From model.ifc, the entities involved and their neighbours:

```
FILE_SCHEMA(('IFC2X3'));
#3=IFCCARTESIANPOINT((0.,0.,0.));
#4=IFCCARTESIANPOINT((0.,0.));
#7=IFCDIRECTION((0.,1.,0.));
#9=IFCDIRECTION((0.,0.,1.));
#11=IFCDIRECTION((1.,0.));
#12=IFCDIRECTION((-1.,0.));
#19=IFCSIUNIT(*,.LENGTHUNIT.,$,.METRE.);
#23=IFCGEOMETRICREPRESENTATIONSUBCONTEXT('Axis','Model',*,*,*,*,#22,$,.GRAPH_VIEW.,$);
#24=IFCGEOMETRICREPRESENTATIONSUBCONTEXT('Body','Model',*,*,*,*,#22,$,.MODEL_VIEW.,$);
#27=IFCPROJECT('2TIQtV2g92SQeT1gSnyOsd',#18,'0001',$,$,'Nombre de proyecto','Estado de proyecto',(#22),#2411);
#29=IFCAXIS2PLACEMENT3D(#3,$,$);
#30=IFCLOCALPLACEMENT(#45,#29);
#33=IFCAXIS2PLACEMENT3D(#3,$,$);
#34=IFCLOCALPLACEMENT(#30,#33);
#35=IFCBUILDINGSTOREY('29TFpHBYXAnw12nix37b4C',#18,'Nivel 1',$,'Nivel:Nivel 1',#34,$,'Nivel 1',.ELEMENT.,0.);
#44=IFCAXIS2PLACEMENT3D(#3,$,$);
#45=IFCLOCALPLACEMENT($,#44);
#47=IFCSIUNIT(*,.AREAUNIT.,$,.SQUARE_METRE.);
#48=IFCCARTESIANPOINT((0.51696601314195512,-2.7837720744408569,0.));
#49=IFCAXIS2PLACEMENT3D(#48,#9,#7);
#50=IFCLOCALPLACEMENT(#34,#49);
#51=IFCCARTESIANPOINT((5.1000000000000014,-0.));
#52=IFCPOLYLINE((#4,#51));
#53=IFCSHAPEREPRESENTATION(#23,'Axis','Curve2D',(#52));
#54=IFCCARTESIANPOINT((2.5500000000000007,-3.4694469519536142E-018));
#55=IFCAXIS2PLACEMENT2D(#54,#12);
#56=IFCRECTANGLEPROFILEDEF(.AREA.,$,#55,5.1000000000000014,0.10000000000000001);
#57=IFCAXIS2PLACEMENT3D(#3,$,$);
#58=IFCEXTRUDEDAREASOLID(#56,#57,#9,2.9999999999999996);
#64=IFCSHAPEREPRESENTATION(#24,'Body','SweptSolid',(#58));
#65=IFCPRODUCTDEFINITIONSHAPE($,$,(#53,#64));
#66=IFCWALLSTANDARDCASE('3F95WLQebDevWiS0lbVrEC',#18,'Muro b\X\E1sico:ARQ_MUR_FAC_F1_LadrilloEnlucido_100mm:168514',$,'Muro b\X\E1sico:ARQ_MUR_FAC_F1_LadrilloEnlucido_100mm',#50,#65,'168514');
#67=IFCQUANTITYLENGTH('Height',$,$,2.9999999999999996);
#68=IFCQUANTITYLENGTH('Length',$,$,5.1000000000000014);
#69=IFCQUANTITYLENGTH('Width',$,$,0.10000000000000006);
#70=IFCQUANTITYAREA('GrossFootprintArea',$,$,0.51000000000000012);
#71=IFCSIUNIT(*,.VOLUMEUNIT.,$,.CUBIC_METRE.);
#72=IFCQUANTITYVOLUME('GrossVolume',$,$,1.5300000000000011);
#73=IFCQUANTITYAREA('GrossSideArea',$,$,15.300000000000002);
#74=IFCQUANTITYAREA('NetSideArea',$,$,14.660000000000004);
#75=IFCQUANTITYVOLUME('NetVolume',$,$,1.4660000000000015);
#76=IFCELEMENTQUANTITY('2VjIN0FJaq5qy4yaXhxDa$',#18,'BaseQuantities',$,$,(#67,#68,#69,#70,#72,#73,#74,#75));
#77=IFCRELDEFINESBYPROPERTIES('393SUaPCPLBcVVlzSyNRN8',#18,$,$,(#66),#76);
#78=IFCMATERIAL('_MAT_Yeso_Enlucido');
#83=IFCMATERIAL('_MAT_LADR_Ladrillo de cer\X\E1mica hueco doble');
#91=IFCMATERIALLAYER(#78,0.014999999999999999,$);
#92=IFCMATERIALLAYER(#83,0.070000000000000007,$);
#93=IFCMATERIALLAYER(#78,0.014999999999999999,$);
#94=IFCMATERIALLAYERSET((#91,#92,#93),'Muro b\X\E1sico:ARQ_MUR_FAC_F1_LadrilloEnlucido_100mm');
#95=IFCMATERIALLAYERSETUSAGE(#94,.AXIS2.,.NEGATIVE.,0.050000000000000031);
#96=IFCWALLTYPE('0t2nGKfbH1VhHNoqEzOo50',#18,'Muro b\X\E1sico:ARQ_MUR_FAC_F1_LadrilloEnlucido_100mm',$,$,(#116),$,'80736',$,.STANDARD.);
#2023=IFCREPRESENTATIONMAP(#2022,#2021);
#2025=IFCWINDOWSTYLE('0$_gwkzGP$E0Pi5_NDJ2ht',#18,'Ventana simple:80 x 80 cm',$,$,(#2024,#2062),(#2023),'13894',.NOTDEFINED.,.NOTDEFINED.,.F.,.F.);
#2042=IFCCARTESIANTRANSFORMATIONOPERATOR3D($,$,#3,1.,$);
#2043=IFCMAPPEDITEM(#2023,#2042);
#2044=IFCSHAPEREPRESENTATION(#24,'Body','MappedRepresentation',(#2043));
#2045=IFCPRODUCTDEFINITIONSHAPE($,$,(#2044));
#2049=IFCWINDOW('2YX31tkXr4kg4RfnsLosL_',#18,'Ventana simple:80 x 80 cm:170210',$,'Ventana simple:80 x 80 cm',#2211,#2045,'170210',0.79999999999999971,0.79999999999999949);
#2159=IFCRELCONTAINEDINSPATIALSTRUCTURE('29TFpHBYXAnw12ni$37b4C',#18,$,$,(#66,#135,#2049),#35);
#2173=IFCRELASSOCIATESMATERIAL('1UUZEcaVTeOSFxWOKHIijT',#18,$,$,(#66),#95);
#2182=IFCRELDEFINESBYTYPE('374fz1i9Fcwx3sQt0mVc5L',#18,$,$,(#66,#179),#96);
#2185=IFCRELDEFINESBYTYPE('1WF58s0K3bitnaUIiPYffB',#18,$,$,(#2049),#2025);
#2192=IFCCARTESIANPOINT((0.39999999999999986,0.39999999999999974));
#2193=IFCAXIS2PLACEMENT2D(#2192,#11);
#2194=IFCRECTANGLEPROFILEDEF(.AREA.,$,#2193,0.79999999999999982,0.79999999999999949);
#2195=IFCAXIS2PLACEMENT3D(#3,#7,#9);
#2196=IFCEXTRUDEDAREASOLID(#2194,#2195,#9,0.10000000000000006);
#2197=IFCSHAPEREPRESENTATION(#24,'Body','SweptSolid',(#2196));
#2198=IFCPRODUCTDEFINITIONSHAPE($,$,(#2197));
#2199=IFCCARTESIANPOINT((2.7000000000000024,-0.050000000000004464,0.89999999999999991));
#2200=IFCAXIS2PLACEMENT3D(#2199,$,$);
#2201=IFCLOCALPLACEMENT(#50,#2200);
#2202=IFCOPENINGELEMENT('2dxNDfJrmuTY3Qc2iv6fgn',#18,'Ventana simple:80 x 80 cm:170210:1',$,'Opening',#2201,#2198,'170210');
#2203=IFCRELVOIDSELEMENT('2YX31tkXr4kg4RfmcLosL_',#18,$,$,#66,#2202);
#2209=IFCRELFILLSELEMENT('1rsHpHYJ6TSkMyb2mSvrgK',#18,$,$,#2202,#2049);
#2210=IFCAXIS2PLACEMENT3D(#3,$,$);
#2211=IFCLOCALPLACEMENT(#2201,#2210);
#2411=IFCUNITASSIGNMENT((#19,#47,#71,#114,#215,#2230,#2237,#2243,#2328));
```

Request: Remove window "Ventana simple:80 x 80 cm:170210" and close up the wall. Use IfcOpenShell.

```python
import ifcopenshell
import ifcopenshell.api.feature
import ifcopenshell.api.pset
import ifcopenshell.api.root
import ifcopenshell.geom
import ifcopenshell.util.element
import ifcopenshell.util.shape
import ifcopenshell.util.unit

model = ifcopenshell.open("model.ifc")
area_scale = ifcopenshell.util.unit.calculate_unit_scale(model, "AREAUNIT")
volume_scale = ifcopenshell.util.unit.calculate_unit_scale(model, "VOLUMEUNIT")
settings = ifcopenshell.geom.settings()


def volume(element):
    """Net volume in cubic metres, openings subtracted."""
    shape = ifcopenshell.geom.create_shape(settings, element)
    return ifcopenshell.util.shape.get_volume(shape.geometry)


window = model.by_id(2049)
opening = window.FillsVoids[0].RelatingOpeningElement
wall = opening.VoidsElements[0].RelatingBuildingElement
before = volume(wall)

ifcopenshell.api.root.remove_product(model, product=window)
ifcopenshell.api.feature.remove_feature(model, feature=opening)

after = volume(wall)
thickness = 0.1  # wall thickness in metres

# Update the wall's stored quantities.
qto = model.by_id(ifcopenshell.util.element.get_pset(wall, "BaseQuantities", should_inherit=False)["id"])
ifcopenshell.api.pset.edit_qto(model, qto=qto, properties={
    "NetSideArea": after / thickness / area_scale,
    "NetVolume": after / volume_scale,
})

print(f"wall volume {before:.3f} -> {after:.3f} m3")

model.write("model_updated.ifc")
```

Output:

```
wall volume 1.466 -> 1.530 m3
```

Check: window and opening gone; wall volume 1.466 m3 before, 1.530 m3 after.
